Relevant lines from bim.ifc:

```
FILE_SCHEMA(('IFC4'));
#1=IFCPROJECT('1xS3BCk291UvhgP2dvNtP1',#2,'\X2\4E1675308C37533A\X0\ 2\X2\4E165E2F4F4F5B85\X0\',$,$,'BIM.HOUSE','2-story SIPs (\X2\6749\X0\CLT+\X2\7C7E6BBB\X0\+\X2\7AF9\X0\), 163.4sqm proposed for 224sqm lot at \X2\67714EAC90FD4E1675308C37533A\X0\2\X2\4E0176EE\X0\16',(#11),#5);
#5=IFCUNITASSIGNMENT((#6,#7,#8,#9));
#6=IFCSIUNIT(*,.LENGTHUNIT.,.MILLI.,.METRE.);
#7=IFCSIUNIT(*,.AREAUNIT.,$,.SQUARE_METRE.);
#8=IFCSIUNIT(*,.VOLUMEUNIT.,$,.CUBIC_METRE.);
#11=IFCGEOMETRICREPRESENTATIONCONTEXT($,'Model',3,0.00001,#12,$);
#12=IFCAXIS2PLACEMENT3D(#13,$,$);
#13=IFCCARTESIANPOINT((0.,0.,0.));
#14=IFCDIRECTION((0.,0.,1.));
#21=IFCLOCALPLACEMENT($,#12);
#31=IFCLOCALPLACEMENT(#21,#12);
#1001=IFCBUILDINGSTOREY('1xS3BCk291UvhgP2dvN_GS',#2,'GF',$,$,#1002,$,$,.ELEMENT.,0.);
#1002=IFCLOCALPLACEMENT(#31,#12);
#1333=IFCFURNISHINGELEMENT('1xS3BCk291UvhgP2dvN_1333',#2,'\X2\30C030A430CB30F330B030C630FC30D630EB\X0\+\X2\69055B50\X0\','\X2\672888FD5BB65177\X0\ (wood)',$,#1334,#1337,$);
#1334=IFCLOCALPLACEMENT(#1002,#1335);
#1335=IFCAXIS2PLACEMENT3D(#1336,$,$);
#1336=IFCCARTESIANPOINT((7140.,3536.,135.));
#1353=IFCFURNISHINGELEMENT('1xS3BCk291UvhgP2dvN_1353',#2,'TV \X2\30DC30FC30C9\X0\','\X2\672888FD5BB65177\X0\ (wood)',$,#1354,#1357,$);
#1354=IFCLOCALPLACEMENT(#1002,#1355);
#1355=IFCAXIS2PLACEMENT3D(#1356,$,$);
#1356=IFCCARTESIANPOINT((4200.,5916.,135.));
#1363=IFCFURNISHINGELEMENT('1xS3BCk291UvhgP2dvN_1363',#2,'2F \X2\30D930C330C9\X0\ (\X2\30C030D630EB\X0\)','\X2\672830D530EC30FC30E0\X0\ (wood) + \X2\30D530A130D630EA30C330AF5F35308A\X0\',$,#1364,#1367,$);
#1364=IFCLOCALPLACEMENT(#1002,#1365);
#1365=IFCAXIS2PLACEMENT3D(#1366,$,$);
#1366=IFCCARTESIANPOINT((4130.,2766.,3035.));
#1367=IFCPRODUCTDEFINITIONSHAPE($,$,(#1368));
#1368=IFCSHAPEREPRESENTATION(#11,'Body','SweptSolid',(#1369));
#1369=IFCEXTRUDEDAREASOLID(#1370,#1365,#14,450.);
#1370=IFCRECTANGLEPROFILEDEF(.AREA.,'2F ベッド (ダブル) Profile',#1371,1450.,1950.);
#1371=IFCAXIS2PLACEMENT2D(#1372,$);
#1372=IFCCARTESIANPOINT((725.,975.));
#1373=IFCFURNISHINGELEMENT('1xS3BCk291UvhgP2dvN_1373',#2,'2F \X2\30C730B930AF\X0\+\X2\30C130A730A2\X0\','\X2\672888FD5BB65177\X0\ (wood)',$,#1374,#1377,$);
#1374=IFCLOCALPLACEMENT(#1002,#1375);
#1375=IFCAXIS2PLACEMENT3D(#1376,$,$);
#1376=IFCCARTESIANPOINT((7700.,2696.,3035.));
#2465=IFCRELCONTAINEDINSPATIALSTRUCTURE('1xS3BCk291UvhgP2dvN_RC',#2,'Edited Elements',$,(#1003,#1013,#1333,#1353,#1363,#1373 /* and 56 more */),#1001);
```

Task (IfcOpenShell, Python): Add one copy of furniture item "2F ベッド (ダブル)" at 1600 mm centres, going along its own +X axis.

```python
import ifcopenshell
import ifcopenshell.api.geometry
import ifcopenshell.api.root
import ifcopenshell.util.element
import ifcopenshell.util.placement

model = ifcopenshell.open("bim.ifc")


def reuse_history(source, copy):
    """copy_class also copies each property set's owner history, people and application; keep the originals."""
    for rel in copy.IsDefinedBy:
        if rel.is_a("IfcRelDefinesByProperties") and (history := rel.RelatingPropertyDefinition.OwnerHistory):
            rel.RelatingPropertyDefinition.OwnerHistory = source.OwnerHistory
            ifcopenshell.util.element.remove_deep2(model, history)


source = model.by_id(1363)
base = ifcopenshell.util.placement.get_local_placement(source.ObjectPlacement)
step = base[:3, 0] * 1600.0

for i in range(1, 2):
    copy = ifcopenshell.api.root.copy_class(model, product=source)
    copy.Representation = ifcopenshell.util.element.copy_deep(
        model, source.Representation, exclude=["IfcGeometricRepresentationContext", "IfcRepresentationMap"]
    )
    reuse_history(source, copy)
    matrix = base.copy()
    matrix[:3, 3] += i * step
    print("added at", matrix[:3, 3].round(3) + 0.0)
    ifcopenshell.api.geometry.edit_object_placement(model, product=copy, matrix=matrix, is_si=False)

model.write("bim-out.ifc")
```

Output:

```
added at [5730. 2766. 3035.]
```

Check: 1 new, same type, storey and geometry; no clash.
